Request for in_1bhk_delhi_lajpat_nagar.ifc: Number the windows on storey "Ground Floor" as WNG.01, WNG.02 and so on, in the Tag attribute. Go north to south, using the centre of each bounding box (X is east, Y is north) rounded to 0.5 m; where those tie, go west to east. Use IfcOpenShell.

First a look at what the model holds.

```python
import ifcopenshell
import ifcopenshell.util.element
import ifcopenshell.util.placement

model = ifcopenshell.open("in_1bhk_delhi_lajpat_nagar.ifc")
print(model.schema)
storey = next(s for s in model.by_type("IfcBuildingStorey") if s.Name == "Ground Floor")
windows = [e for e in ifcopenshell.util.element.get_decomposition(storey) if e.is_a("IfcWindow")]
for e in sorted(windows, key=lambda e: e.id()):
    origin = ifcopenshell.util.placement.get_local_placement(e.ObjectPlacement)[:3, 3]
    print(e.id(), e.Tag, e.Name, origin.round(2) + 0.0, sep=" | ")
```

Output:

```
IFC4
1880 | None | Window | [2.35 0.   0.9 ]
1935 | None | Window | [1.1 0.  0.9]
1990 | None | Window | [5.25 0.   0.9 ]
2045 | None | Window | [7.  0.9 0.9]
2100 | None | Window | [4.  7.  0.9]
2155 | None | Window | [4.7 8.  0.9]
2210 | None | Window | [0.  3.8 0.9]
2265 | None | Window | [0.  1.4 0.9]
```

```python
import ifcopenshell
import ifcopenshell.geom
import ifcopenshell.util.element
import ifcopenshell.util.shape

model = ifcopenshell.open("in_1bhk_delhi_lajpat_nagar.ifc")
settings = ifcopenshell.geom.settings()
settings.set("use-world-coords", True)


def centre(element):
    shape = ifcopenshell.geom.create_shape(settings, element)
    return ifcopenshell.util.shape.get_bbox_centroid(shape.geometry)


storey = next(s for s in model.by_type("IfcBuildingStorey") if s.Name == "Ground Floor")
windows = [e for e in ifcopenshell.util.element.get_decomposition(storey) if e.is_a("IfcWindow")]

# Insertion points can sit at a corner or the storey origin, so sort by the geometry (in metres).
centres = {e: centre(e) for e in windows}
windows.sort(key=lambda e: (-round(centres[e][1] / 0.5), centres[e][0]))

for i, e in enumerate(windows, start=1):
    number = f"WNG.{i:02d}"
    e.Tag = number
    print(e.id(), number)

model.write("in_1bhk_delhi_lajpat_nagar_edited.ifc")
```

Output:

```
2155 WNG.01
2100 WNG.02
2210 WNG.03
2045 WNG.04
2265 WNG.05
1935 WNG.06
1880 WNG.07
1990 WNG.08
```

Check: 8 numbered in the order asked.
